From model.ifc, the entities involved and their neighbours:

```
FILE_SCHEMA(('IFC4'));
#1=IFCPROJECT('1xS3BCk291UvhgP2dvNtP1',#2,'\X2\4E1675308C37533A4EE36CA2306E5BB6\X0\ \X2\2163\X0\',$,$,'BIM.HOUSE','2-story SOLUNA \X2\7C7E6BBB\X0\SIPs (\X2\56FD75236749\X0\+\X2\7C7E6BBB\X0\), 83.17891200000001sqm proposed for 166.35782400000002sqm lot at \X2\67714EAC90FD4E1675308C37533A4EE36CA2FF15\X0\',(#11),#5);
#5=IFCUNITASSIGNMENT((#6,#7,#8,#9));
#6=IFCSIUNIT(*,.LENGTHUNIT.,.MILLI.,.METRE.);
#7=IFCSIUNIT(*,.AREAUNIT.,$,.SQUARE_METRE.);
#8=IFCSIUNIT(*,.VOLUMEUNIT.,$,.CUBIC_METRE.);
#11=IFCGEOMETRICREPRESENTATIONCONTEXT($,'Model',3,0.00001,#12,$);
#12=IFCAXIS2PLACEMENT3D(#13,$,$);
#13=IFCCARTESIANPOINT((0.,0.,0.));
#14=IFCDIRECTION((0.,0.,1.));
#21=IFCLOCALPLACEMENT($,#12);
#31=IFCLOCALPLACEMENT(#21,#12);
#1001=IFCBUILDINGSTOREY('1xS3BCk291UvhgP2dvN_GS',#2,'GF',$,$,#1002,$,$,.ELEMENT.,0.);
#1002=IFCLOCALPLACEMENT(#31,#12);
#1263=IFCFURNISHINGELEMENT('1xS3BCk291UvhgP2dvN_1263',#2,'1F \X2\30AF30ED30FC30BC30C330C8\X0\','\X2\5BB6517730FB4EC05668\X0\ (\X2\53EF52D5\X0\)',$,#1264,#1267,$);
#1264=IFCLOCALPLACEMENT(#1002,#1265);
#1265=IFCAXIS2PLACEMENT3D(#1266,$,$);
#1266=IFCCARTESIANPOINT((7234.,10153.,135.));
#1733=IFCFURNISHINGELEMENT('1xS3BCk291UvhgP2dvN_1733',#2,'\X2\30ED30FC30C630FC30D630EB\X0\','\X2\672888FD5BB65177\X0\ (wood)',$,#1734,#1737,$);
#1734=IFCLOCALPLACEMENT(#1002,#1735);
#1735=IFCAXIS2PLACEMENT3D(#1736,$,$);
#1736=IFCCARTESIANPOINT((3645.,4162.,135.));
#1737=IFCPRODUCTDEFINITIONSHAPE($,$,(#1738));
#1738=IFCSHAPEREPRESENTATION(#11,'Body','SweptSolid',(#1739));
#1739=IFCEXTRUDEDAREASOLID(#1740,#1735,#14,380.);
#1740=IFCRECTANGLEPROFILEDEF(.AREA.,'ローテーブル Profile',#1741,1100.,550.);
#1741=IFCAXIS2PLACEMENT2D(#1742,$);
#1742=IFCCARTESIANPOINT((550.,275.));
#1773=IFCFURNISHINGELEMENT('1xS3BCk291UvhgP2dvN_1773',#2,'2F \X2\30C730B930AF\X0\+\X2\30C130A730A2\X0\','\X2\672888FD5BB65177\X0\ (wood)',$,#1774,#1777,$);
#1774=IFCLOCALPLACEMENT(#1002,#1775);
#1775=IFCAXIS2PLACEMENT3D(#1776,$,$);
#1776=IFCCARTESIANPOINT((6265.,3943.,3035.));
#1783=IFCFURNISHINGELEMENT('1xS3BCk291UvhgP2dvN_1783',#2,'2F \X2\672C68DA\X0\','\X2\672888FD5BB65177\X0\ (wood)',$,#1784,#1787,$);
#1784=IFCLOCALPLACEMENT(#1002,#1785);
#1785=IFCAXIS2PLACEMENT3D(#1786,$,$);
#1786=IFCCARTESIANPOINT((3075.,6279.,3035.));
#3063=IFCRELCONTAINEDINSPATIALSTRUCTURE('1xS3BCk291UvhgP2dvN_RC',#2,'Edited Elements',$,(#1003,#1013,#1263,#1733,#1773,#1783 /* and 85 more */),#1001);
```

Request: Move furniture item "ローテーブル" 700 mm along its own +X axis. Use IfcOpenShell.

```python
import ifcopenshell
import ifcopenshell.api.geometry
import ifcopenshell.util.placement

model = ifcopenshell.open("model.ifc")

item = model.by_guid("1xS3BCk291UvhgP2dvN_1733")
matrix = ifcopenshell.util.placement.get_local_placement(item.ObjectPlacement)
matrix[:3, 3] += matrix[:3, 0] * 700.0
ifcopenshell.api.geometry.edit_object_placement(model, product=item, matrix=matrix, is_si=False)

print(ifcopenshell.util.placement.get_local_placement(item.ObjectPlacement).round(3) + 0.0)

model.write("model-out.ifc")
```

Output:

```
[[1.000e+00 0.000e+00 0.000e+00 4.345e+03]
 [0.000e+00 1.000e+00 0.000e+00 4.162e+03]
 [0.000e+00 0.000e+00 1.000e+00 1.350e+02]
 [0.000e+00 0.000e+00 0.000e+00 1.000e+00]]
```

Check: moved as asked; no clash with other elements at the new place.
